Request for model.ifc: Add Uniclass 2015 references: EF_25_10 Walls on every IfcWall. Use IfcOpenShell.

First a look at what the model holds.

```python
import ifcopenshell

model = ifcopenshell.open("model.ifc")
print(model.schema)
print("classifications:", [c.Name for c in model.by_type("IfcClassification")])
for ifc_class in ("IfcDoor", "IfcRoof", "IfcStair", "IfcWall", "IfcWindow"):
    print(ifc_class, len(model.by_type(ifc_class)))
```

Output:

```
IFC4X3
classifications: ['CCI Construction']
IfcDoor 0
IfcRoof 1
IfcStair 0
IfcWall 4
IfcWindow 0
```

```python
import ifcopenshell
import ifcopenshell.api.classification

model = ifcopenshell.open("model.ifc")

system = ifcopenshell.api.classification.add_classification(model, classification="Uniclass 2015")

codes = {
    "IfcWall": ("EF_25_10", "Walls"),
}
for ifc_class, (code, name) in codes.items():
    products = model.by_type(ifc_class)
    ifcopenshell.api.classification.add_reference(
        model, products=products, classification=system, identification=code, name=name
    )
    print(code, len(products))

model.write("model_v2.ifc")
```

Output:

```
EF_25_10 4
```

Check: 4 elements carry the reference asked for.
